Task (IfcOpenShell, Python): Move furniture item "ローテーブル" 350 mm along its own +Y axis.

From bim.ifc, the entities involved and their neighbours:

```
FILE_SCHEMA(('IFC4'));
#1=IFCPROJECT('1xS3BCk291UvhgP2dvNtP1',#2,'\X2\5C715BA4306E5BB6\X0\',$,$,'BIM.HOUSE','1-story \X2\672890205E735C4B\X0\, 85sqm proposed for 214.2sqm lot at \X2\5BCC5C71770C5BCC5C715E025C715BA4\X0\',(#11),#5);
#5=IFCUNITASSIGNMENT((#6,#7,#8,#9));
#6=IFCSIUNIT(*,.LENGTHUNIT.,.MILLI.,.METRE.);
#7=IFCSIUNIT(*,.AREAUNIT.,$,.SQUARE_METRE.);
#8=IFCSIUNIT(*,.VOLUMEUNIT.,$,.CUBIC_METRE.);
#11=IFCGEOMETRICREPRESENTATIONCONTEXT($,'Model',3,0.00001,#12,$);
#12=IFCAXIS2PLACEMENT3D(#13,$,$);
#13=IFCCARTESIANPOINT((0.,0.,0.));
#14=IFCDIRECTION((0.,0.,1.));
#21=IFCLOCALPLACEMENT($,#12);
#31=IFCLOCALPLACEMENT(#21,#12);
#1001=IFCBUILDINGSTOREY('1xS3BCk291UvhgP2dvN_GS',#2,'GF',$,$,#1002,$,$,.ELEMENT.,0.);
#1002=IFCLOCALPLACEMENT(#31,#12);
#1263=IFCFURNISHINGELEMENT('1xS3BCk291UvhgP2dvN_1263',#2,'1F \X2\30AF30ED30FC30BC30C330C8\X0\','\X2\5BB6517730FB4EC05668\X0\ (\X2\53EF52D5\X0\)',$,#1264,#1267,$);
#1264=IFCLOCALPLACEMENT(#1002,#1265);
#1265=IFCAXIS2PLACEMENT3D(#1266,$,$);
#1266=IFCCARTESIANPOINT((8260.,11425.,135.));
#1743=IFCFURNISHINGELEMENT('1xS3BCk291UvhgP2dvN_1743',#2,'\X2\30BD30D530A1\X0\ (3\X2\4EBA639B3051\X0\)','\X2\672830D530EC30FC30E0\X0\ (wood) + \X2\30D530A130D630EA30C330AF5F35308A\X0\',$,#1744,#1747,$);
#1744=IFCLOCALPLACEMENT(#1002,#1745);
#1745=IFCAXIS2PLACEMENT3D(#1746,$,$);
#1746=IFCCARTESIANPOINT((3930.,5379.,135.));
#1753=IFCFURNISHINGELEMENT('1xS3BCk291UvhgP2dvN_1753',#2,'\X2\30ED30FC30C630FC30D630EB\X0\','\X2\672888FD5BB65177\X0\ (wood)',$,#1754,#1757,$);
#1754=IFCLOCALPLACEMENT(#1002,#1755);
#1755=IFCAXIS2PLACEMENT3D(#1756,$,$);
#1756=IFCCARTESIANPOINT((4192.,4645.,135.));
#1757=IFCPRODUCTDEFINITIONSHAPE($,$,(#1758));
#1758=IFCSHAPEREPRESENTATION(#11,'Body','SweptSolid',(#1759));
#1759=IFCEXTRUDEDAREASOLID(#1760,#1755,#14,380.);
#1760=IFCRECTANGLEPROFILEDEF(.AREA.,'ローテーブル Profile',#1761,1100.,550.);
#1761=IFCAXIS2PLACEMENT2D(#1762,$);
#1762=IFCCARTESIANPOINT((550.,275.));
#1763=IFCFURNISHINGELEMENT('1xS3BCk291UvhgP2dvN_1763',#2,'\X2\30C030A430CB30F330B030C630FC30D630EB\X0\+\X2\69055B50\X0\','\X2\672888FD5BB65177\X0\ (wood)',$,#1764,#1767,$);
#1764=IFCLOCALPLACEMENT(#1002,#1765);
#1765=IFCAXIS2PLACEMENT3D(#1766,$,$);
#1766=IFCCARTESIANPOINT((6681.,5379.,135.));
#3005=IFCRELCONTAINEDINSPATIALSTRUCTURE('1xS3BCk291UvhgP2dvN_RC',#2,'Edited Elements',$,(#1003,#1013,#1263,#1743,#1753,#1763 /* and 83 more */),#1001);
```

```python
import ifcopenshell
import ifcopenshell.api.geometry
import ifcopenshell.util.placement
import ifcopenshell.util.unit

model = ifcopenshell.open("bim.ifc")
unit_scale = ifcopenshell.util.unit.calculate_unit_scale(model)

item = model.by_id(1753)
matrix = ifcopenshell.util.placement.get_local_placement(item.ObjectPlacement)
matrix[:3, 3] += matrix[:3, 1] * 0.35 / unit_scale
ifcopenshell.api.geometry.edit_object_placement(model, product=item, matrix=matrix, is_si=False)

print(ifcopenshell.util.placement.get_local_placement(item.ObjectPlacement).round(3) + 0.0)

model.write("bim_v2.ifc")
```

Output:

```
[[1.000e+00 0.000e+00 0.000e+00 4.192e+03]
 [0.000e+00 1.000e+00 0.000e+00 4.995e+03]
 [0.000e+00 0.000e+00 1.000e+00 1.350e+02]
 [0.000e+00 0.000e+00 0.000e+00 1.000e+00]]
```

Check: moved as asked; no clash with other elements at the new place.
